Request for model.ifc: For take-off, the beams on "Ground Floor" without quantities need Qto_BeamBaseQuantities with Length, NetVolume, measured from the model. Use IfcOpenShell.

First a look at what the model holds.

```python
import ifcopenshell
import ifcopenshell.util.element
import ifcopenshell.util.unit

model = ifcopenshell.open("model.ifc")
print(model.schema)
for unit_type in ("LENGTHUNIT", "AREAUNIT", "VOLUMEUNIT"):
    print(unit_type, ifcopenshell.util.unit.calculate_unit_scale(model, unit_type))
storey = next(s for s in model.by_type("IfcBuildingStorey") if s.Name == "Ground Floor")
beams = [e for e in ifcopenshell.util.element.get_decomposition(storey) if e.is_a("IfcBeam")]
for e in sorted(beams, key=lambda e: e.id()):
    print(e.id(), e.is_a(), e.Name, list(ifcopenshell.util.element.get_psets(e, qtos_only=True)), sep=" | ")
```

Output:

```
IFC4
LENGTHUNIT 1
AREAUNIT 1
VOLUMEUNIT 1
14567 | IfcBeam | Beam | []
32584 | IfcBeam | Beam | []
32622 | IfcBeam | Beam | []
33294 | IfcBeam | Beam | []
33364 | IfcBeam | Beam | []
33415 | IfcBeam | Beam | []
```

```python
import ifcopenshell
import ifcopenshell.api.pset
import ifcopenshell.geom
import ifcopenshell.util.element
import ifcopenshell.util.shape
import ifcopenshell.util.unit

model = ifcopenshell.open("model.ifc")
unit_scale = ifcopenshell.util.unit.calculate_unit_scale(model)
volume_scale = ifcopenshell.util.unit.calculate_unit_scale(model, "VOLUMEUNIT")
settings = ifcopenshell.geom.settings()

storey = next(s for s in model.by_type("IfcBuildingStorey") if s.Name == "Ground Floor")
beams = [e for e in ifcopenshell.util.element.get_decomposition(storey) if e.is_a("IfcBeam")]

for e in sorted(beams, key=lambda e: e.id()):
    if ifcopenshell.util.element.get_psets(e, qtos_only=True, should_inherit=False):
        continue
    # Geometry comes back in metres, in the element's own axes.
    shape = ifcopenshell.geom.create_shape(settings, e)
    values = {
        "Length": ifcopenshell.util.shape.get_max_xyz(shape.geometry) / unit_scale,
        "NetVolume": ifcopenshell.util.shape.get_volume(shape.geometry) / volume_scale,
    }
    qto = ifcopenshell.api.pset.add_qto(model, product=e, name="Qto_BeamBaseQuantities")
    ifcopenshell.api.pset.edit_qto(model, qto=qto, properties=values)
    print(e.id(), {k: round(v, 3) for k, v in values.items()})

model.write("model_v2.ifc")
```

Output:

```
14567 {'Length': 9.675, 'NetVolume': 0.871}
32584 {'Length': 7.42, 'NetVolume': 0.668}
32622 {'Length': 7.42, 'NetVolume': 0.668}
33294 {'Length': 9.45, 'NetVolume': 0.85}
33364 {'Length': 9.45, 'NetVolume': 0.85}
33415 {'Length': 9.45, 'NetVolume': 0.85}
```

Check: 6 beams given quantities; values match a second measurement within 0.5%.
